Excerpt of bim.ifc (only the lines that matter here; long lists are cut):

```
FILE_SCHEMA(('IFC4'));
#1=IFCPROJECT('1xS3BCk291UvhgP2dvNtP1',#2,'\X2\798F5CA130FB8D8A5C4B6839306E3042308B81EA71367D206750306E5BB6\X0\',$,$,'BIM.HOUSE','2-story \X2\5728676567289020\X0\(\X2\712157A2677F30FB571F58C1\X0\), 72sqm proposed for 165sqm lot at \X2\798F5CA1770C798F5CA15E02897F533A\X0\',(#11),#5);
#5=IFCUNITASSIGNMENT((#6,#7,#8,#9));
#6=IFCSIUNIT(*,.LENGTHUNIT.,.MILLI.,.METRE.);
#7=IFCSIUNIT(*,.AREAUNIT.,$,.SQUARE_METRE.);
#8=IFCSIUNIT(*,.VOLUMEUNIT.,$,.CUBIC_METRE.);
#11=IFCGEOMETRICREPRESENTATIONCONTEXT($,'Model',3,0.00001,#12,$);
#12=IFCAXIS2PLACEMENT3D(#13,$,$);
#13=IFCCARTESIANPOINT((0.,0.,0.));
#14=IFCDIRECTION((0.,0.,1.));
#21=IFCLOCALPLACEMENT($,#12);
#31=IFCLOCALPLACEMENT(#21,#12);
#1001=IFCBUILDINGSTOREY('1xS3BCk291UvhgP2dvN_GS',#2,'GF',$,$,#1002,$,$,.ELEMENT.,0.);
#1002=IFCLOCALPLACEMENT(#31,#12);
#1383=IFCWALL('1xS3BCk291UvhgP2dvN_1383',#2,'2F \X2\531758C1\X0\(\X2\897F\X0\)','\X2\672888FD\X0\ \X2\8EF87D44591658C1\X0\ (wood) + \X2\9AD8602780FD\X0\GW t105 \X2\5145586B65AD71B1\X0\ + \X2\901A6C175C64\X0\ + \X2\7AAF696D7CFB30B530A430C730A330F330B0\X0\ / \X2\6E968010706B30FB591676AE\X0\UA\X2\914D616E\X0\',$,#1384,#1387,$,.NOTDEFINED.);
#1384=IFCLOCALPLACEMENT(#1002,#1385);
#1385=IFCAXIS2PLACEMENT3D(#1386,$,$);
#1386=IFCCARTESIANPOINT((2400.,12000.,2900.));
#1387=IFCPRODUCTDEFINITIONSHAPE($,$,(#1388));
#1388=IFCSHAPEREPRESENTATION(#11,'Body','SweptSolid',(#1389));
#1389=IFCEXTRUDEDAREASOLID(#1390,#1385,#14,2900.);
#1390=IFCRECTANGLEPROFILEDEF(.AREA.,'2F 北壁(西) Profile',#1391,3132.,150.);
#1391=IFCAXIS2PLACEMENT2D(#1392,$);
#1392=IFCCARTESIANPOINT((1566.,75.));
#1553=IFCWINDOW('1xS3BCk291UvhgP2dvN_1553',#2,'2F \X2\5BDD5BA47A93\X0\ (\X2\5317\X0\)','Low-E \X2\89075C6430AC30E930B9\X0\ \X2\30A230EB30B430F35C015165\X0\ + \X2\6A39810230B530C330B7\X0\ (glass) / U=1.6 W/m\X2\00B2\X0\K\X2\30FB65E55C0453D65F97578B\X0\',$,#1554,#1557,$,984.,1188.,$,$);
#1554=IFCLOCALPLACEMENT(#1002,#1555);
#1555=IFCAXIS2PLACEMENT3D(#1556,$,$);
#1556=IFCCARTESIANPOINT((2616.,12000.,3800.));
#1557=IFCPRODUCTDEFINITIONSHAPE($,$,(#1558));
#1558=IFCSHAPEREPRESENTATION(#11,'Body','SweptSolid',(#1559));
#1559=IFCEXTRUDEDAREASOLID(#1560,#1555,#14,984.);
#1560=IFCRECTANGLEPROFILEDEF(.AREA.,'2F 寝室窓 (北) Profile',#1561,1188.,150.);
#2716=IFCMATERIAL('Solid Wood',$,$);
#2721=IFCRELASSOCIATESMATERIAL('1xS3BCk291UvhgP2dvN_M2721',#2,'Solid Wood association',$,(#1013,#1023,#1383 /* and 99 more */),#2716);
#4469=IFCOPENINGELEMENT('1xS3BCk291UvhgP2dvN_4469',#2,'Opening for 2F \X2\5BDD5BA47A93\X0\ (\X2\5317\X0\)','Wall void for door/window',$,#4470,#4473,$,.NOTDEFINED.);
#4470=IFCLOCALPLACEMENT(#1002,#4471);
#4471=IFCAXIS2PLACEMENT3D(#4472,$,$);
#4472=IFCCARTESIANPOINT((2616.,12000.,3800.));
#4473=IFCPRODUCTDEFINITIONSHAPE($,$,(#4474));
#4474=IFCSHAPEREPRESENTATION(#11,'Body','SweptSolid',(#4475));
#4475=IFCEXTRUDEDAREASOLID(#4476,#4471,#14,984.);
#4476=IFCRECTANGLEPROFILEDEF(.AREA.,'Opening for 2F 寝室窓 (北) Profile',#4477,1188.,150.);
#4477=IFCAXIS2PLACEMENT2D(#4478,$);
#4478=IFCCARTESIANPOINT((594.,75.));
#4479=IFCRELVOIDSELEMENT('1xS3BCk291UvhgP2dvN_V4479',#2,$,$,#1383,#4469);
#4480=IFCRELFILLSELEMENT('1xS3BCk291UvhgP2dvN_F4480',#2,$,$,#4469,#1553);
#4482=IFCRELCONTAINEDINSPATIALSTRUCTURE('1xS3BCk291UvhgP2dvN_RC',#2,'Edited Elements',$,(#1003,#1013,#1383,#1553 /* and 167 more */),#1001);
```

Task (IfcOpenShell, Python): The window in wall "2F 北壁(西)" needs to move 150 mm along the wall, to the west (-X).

```python
import ifcopenshell
import ifcopenshell.api.geometry
import ifcopenshell.util.placement
import ifcopenshell.util.unit

model = ifcopenshell.open("bim.ifc")
unit_scale = ifcopenshell.util.unit.calculate_unit_scale(model)

window = model.by_guid("1xS3BCk291UvhgP2dvN_1553")
opening = window.FillsVoids[0].RelatingOpeningElement
wall = opening.VoidsElements[0].RelatingBuildingElement

wall_matrix = ifcopenshell.util.placement.get_local_placement(wall.ObjectPlacement)
shift = wall_matrix[:3, 0] * -0.15 / unit_scale
before = ifcopenshell.util.placement.get_local_placement(window.ObjectPlacement)[:3, 3].copy()

# The window is not placed relative to its opening, so move both.
for product in (opening, window):
    matrix = ifcopenshell.util.placement.get_local_placement(product.ObjectPlacement)
    matrix[:3, 3] += shift
    ifcopenshell.api.geometry.edit_object_placement(model, product=product, matrix=matrix, is_si=False)

after = ifcopenshell.util.placement.get_local_placement(window.ObjectPlacement)[:3, 3]
print("window moved by", (after - before).round(3) + 0.0)

model.write("bim-out.ifc")
```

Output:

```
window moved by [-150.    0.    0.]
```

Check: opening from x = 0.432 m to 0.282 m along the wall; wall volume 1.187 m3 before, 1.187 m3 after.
